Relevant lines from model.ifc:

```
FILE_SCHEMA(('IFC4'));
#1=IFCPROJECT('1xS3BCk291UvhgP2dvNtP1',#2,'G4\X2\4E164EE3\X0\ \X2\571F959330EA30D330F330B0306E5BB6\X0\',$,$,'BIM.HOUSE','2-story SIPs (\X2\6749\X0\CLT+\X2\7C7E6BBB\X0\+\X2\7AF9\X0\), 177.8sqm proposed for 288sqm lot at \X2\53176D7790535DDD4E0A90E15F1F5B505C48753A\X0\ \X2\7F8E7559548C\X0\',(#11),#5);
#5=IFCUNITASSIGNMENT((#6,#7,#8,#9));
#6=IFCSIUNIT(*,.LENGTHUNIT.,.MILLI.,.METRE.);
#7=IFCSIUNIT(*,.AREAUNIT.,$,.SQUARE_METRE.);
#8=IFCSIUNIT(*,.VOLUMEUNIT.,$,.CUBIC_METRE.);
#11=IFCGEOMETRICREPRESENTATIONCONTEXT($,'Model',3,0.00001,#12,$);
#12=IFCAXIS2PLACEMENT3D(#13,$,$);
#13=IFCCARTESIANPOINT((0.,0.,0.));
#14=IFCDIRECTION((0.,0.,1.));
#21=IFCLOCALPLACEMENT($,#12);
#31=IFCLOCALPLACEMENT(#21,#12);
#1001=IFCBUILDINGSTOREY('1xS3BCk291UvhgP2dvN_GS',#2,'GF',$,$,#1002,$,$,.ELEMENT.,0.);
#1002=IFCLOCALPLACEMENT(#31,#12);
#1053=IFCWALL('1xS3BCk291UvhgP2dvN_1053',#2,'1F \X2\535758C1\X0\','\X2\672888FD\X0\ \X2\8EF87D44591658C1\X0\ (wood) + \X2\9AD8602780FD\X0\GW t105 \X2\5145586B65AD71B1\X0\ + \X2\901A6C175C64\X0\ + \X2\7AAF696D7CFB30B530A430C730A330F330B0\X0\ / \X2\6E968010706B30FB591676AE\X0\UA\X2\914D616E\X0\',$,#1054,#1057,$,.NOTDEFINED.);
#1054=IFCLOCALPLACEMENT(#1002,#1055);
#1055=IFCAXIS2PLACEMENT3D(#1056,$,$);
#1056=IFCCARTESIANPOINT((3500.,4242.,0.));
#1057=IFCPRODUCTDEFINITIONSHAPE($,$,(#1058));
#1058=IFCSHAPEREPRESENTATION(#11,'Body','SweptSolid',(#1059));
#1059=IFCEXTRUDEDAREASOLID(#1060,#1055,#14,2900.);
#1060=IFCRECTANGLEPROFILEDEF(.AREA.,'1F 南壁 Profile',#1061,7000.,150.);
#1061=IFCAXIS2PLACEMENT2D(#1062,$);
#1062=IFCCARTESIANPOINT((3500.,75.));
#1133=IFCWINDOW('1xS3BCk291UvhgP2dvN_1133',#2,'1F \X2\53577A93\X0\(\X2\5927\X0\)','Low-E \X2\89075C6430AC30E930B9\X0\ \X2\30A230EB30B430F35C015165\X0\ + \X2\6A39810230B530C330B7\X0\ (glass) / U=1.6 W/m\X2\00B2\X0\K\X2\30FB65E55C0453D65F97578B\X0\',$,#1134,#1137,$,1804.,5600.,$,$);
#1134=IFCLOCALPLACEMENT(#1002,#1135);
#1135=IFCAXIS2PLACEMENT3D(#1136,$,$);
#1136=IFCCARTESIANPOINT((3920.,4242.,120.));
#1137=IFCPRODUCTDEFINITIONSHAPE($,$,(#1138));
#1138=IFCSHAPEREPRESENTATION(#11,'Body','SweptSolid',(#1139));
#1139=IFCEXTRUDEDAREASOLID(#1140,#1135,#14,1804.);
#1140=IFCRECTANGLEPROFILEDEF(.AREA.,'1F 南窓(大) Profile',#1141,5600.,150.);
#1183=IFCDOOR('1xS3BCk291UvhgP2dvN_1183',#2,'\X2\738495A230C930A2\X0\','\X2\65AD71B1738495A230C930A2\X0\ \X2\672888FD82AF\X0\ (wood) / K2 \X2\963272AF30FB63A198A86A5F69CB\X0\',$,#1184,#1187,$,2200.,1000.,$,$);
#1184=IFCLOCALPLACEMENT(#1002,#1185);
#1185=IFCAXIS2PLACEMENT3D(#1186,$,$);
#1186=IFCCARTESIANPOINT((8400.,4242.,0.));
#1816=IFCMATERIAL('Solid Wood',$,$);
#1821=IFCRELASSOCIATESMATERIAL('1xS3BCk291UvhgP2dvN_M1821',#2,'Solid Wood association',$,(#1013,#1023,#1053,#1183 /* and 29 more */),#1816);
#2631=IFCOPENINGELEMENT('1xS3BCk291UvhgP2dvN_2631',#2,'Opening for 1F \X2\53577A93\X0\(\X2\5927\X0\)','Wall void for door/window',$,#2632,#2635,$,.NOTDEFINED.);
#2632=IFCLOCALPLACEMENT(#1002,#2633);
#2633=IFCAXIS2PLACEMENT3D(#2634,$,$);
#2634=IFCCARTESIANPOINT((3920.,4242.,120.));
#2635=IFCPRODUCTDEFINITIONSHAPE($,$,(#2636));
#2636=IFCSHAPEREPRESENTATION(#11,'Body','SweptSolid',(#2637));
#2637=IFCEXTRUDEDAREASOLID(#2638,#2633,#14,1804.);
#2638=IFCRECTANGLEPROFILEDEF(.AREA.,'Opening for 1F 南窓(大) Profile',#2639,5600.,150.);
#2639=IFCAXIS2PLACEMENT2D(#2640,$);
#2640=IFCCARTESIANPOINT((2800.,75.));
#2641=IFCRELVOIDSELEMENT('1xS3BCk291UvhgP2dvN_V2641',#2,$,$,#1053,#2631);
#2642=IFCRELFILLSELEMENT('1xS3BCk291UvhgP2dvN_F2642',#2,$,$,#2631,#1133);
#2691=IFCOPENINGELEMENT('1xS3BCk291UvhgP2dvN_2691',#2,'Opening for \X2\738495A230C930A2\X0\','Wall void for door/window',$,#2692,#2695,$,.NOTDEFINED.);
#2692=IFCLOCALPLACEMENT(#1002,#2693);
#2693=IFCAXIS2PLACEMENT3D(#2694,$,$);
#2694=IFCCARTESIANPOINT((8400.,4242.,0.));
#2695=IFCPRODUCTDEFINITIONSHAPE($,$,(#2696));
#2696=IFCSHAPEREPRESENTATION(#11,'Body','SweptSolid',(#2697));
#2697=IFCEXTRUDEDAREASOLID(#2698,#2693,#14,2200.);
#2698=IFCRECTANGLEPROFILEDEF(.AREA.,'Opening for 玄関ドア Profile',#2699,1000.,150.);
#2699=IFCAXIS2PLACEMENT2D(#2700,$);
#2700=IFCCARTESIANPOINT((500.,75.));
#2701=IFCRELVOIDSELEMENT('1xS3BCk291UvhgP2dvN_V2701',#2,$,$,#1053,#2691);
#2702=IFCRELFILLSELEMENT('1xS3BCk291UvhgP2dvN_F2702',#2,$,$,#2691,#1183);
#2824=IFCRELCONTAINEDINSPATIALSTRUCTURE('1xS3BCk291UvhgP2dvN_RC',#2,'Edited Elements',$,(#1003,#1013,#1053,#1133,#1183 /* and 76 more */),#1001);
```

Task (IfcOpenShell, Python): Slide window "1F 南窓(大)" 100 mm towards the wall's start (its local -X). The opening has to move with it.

```python
import ifcopenshell
import ifcopenshell.api.geometry
import ifcopenshell.util.placement
import ifcopenshell.util.unit

model = ifcopenshell.open("model.ifc")
unit_scale = ifcopenshell.util.unit.calculate_unit_scale(model)

window = model.by_id(1133)
opening = window.FillsVoids[0].RelatingOpeningElement
wall = opening.VoidsElements[0].RelatingBuildingElement

wall_matrix = ifcopenshell.util.placement.get_local_placement(wall.ObjectPlacement)
shift = wall_matrix[:3, 0] * -0.1 / unit_scale
before = ifcopenshell.util.placement.get_local_placement(window.ObjectPlacement)[:3, 3].copy()

# The window is not placed relative to its opening, so move both.
for product in (opening, window):
    matrix = ifcopenshell.util.placement.get_local_placement(product.ObjectPlacement)
    matrix[:3, 3] += shift
    ifcopenshell.api.geometry.edit_object_placement(model, product=product, matrix=matrix, is_si=False)

after = ifcopenshell.util.placement.get_local_placement(window.ObjectPlacement)[:3, 3]
print("window moved by", (after - before).round(3) + 0.0)

model.write("model_v2.ifc")
```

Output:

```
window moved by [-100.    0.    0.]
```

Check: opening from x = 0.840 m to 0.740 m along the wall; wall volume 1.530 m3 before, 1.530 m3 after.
